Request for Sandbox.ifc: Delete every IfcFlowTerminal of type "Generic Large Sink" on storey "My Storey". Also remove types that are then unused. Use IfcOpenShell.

First a look at what the model holds.

```python
import ifcopenshell
import ifcopenshell.util.element

model = ifcopenshell.open("Sandbox.ifc")
print(model.schema)
storey = next(s for s in model.by_type("IfcBuildingStorey") if s.Name == "My Storey")
terminals = [e for e in ifcopenshell.util.element.get_decomposition(storey) if e.is_a("IfcFlowTerminal")]
seen = {}
for e in terminals:
    element_type = ifcopenshell.util.element.get_type(e)
    name = element_type.Name if element_type not in (None, e) else None
    seen[name] = seen.get(name, 0) + 1
for name, count in sorted(seen.items(), key=str):
    print(count, "x", name)
```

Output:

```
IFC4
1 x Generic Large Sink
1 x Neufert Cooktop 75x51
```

```python
import ifcopenshell
import ifcopenshell.api.root
import ifcopenshell.util.element

model = ifcopenshell.open("Sandbox.ifc")

storey = next(s for s in model.by_type("IfcBuildingStorey") if s.Name == "My Storey")
terminals = [e for e in ifcopenshell.util.element.get_decomposition(storey) if e.is_a("IfcFlowTerminal")]
targets = [e for e in terminals if (t := ifcopenshell.util.element.get_type(e)) not in (None, e) and t.Name == "Generic Large Sink"]
types = {ifcopenshell.util.element.get_type(e) for e in targets} - {None, *targets}

for e in targets:
    ifcopenshell.api.root.remove_product(model, product=e)
print(len(targets), "removed")

unused = [t for t in types if not ifcopenshell.util.element.get_types(t)]
for t in unused:
    ifcopenshell.api.root.remove_product(model, product=t)
print(len(unused), "unused types removed")

model.write("Sandbox_edited.ifc")
```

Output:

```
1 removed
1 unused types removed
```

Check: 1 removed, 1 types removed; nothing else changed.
